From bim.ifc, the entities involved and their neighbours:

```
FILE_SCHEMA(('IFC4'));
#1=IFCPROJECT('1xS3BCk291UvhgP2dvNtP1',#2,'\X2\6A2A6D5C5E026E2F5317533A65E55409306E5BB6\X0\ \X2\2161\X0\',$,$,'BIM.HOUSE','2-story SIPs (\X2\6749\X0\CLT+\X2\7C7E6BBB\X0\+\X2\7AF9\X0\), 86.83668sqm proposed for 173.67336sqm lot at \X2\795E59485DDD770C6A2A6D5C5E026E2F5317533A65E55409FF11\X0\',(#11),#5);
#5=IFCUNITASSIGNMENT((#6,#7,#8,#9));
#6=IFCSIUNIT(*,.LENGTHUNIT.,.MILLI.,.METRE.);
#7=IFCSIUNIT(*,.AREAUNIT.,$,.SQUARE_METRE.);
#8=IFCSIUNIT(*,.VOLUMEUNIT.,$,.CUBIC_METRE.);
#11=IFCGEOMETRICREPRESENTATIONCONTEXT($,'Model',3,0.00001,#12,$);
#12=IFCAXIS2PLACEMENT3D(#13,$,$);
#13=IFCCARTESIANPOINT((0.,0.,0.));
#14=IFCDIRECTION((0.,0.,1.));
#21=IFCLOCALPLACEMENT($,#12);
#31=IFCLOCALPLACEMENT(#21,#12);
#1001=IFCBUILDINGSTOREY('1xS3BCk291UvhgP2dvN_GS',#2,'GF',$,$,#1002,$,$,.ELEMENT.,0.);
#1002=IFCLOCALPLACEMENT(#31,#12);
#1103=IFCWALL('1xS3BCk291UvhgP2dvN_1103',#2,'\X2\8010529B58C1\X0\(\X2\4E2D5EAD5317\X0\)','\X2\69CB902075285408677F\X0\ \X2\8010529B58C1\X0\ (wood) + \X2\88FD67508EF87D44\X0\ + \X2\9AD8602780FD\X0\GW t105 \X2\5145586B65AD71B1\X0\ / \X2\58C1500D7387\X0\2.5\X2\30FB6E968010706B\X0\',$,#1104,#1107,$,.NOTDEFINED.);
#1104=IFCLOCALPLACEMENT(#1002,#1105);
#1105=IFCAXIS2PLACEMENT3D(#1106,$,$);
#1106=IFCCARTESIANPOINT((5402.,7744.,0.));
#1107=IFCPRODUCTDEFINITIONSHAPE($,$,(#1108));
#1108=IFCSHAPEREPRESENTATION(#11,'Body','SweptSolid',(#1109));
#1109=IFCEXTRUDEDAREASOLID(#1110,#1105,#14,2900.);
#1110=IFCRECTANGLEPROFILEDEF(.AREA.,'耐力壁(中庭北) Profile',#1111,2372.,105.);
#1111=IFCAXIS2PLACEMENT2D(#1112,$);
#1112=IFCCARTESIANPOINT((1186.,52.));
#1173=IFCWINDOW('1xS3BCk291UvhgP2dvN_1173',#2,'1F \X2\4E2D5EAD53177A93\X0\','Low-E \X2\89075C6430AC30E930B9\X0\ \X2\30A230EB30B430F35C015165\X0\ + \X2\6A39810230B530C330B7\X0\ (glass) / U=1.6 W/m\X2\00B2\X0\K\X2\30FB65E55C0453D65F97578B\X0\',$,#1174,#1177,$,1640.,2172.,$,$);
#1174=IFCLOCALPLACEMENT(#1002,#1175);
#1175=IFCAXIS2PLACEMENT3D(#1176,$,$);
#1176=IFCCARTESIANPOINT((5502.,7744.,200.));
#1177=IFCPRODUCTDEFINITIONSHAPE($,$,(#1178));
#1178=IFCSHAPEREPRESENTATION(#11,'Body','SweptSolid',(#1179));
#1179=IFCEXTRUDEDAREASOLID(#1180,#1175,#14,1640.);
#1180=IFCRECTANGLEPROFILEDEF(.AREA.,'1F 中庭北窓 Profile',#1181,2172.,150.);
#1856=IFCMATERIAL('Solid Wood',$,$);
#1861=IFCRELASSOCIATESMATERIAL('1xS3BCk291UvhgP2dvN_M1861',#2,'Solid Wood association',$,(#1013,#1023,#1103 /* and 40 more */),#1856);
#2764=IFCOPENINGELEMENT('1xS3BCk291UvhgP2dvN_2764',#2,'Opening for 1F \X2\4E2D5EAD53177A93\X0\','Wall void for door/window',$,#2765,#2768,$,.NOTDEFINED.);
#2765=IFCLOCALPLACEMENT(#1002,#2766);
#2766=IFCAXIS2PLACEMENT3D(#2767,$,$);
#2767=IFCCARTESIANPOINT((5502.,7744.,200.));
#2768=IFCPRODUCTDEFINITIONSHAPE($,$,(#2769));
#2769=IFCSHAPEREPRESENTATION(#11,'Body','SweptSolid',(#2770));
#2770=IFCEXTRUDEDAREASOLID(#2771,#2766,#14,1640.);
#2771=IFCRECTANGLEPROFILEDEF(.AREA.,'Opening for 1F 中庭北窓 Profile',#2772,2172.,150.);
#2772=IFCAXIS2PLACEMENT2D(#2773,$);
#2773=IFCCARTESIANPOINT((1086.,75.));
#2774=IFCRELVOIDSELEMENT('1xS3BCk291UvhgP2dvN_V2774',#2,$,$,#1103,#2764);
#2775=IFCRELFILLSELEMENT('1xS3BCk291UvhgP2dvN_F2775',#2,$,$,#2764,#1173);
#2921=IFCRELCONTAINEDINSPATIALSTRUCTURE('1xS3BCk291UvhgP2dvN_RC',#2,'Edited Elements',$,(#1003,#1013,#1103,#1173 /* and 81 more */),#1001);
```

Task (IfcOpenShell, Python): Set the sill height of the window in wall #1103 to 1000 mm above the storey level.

```python
import numpy as np
import ifcopenshell
import ifcopenshell.api.geometry
import ifcopenshell.geom
import ifcopenshell.util.element
import ifcopenshell.util.placement
import ifcopenshell.util.shape
import ifcopenshell.util.unit

model = ifcopenshell.open("bim.ifc")
unit_scale = ifcopenshell.util.unit.calculate_unit_scale(model)

window = model.by_id(1173)
opening = window.FillsVoids[0].RelatingOpeningElement
storey = ifcopenshell.util.element.get_container(window, ifc_class="IfcBuildingStorey")
level = ifcopenshell.util.placement.get_local_placement(storey.ObjectPlacement)[2, 3]

# The opening's origin need not be at the sill, so measure its lowest point.
shape = ifcopenshell.geom.create_shape(ifcopenshell.geom.settings(), opening)
bottom = ifcopenshell.util.shape.get_shape_bottom_elevation(shape, shape.geometry) / unit_scale
dz = level + 1 / unit_scale - bottom

shift = np.array([0.0, 0.0, dz])
# The window is not placed relative to its opening, so move both.
for product in (opening, window):
    matrix = ifcopenshell.util.placement.get_local_placement(product.ObjectPlacement)
    matrix[:3, 3] += shift
    ifcopenshell.api.geometry.edit_object_placement(model, product=product, matrix=matrix, is_si=False)

print(f"moved by {dz * unit_scale:+.3f} m")

model.write("bim_rev.ifc")
```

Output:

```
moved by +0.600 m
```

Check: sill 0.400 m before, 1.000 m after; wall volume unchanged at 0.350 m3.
